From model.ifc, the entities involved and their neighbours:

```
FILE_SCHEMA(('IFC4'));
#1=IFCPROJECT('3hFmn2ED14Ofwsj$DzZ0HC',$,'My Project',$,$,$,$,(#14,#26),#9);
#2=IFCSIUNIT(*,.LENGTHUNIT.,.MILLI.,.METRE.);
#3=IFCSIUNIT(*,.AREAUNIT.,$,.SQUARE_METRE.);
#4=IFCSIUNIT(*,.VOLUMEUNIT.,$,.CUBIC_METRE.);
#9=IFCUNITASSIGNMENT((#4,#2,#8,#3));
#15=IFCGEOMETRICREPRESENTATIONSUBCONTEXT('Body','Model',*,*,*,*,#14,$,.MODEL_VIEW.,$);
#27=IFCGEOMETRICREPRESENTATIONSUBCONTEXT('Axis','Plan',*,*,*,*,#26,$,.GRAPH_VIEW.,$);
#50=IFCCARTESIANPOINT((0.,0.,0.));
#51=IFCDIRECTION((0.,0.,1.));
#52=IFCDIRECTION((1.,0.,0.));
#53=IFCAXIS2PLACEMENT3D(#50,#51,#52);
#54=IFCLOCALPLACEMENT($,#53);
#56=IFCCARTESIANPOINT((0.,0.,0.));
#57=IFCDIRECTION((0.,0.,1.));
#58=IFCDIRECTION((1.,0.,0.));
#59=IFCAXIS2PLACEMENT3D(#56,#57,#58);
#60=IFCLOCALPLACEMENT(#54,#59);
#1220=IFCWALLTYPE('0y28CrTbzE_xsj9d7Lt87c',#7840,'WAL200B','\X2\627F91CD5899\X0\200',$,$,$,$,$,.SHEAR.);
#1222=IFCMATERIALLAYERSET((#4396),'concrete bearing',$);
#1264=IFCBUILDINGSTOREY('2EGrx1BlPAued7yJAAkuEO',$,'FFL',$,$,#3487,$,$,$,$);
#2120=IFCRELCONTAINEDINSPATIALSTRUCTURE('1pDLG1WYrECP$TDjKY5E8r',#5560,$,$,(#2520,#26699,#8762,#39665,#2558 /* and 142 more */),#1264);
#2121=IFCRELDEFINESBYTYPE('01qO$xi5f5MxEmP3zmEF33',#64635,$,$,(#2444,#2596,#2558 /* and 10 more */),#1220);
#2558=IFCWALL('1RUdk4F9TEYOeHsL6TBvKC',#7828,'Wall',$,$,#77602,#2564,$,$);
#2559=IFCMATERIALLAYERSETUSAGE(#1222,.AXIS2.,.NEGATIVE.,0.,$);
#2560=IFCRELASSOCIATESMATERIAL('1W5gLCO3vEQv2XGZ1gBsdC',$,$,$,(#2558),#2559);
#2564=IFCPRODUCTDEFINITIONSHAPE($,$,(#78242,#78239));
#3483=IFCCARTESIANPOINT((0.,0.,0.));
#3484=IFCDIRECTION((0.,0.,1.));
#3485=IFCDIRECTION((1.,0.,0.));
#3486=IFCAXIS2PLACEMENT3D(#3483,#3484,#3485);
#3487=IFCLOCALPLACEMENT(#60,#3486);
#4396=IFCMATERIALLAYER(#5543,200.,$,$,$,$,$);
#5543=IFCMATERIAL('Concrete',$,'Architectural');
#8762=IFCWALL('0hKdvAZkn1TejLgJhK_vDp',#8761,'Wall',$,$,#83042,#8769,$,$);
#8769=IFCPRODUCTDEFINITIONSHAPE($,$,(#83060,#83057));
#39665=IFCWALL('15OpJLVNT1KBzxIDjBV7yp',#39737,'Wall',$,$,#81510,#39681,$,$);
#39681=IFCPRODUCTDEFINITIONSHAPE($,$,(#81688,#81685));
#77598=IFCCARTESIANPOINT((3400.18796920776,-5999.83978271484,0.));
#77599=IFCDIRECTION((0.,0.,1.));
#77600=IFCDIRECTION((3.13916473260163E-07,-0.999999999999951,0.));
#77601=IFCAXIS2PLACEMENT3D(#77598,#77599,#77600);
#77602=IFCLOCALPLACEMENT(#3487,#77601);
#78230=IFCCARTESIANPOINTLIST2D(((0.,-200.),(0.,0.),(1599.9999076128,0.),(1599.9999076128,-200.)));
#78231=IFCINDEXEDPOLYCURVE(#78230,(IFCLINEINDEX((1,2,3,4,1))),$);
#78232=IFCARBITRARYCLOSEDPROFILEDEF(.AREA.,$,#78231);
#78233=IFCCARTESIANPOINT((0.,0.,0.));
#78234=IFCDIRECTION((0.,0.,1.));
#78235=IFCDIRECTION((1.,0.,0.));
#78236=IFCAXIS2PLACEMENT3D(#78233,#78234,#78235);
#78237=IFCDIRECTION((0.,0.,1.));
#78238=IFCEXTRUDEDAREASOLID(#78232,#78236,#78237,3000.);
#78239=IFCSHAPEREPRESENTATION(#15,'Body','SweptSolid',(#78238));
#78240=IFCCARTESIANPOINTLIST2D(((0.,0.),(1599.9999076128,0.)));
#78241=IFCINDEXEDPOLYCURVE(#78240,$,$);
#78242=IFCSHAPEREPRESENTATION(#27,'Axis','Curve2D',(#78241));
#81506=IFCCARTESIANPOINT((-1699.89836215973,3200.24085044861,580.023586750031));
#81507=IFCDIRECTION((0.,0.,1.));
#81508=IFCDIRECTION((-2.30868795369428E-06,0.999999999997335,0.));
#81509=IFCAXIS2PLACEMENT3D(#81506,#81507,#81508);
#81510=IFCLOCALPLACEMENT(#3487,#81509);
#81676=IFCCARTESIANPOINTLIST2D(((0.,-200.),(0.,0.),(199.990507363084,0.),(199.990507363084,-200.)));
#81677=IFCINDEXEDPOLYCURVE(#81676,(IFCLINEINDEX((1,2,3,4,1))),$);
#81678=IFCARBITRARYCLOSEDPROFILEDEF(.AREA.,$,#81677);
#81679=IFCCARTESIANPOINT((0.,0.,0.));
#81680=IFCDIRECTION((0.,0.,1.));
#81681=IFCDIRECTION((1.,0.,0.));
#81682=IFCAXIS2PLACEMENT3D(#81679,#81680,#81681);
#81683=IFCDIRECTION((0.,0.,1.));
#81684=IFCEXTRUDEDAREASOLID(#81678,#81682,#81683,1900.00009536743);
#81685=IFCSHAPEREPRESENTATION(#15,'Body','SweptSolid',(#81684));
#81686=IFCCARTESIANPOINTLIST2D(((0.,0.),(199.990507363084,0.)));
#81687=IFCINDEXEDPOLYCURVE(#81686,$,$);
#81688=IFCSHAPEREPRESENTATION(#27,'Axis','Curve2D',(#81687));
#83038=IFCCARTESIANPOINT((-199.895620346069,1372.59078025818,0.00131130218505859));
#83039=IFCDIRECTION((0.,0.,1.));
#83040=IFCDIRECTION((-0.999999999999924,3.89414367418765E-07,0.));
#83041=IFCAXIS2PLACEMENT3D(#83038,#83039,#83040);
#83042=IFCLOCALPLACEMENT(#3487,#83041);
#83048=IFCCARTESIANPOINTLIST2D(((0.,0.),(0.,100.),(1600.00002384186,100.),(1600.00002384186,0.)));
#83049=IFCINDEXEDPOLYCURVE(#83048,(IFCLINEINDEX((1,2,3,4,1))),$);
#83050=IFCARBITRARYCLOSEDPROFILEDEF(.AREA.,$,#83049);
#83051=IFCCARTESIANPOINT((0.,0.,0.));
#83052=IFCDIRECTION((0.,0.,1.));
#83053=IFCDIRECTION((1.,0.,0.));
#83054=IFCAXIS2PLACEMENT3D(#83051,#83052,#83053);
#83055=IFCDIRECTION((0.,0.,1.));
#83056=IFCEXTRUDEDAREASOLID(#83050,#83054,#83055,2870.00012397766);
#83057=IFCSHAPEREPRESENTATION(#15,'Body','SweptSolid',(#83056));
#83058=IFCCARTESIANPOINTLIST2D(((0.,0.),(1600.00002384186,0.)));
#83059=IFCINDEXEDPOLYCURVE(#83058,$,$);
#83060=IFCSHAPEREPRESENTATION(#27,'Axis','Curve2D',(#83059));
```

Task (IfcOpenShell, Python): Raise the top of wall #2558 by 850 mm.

```python
import ifcopenshell
import ifcopenshell.geom
import ifcopenshell.util.representation
import ifcopenshell.util.shape
import ifcopenshell.util.unit

model = ifcopenshell.open("model.ifc")
unit_scale = ifcopenshell.util.unit.calculate_unit_scale(model)
settings = ifcopenshell.geom.settings()


def volume(element):
    """Net volume in cubic metres, openings subtracted."""
    shape = ifcopenshell.geom.create_shape(settings, element)
    return ifcopenshell.util.shape.get_volume(shape.geometry)


wall = model.by_guid("1RUdk4F9TEYOeHsL6TBvKC")
before = volume(wall)

body = ifcopenshell.util.representation.get_representation(wall, "Model", "Body")
solid = body.Items[0]
old_height = solid.Depth
solid.Depth += 0.85 / unit_scale
after = volume(wall)

print(f"height {old_height:g} -> {solid.Depth:g}, volume {before:.3f} -> {after:.3f} m3")

model.write("model_v2.ifc")
```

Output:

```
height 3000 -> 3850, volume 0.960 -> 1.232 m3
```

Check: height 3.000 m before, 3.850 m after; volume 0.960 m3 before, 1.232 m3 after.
